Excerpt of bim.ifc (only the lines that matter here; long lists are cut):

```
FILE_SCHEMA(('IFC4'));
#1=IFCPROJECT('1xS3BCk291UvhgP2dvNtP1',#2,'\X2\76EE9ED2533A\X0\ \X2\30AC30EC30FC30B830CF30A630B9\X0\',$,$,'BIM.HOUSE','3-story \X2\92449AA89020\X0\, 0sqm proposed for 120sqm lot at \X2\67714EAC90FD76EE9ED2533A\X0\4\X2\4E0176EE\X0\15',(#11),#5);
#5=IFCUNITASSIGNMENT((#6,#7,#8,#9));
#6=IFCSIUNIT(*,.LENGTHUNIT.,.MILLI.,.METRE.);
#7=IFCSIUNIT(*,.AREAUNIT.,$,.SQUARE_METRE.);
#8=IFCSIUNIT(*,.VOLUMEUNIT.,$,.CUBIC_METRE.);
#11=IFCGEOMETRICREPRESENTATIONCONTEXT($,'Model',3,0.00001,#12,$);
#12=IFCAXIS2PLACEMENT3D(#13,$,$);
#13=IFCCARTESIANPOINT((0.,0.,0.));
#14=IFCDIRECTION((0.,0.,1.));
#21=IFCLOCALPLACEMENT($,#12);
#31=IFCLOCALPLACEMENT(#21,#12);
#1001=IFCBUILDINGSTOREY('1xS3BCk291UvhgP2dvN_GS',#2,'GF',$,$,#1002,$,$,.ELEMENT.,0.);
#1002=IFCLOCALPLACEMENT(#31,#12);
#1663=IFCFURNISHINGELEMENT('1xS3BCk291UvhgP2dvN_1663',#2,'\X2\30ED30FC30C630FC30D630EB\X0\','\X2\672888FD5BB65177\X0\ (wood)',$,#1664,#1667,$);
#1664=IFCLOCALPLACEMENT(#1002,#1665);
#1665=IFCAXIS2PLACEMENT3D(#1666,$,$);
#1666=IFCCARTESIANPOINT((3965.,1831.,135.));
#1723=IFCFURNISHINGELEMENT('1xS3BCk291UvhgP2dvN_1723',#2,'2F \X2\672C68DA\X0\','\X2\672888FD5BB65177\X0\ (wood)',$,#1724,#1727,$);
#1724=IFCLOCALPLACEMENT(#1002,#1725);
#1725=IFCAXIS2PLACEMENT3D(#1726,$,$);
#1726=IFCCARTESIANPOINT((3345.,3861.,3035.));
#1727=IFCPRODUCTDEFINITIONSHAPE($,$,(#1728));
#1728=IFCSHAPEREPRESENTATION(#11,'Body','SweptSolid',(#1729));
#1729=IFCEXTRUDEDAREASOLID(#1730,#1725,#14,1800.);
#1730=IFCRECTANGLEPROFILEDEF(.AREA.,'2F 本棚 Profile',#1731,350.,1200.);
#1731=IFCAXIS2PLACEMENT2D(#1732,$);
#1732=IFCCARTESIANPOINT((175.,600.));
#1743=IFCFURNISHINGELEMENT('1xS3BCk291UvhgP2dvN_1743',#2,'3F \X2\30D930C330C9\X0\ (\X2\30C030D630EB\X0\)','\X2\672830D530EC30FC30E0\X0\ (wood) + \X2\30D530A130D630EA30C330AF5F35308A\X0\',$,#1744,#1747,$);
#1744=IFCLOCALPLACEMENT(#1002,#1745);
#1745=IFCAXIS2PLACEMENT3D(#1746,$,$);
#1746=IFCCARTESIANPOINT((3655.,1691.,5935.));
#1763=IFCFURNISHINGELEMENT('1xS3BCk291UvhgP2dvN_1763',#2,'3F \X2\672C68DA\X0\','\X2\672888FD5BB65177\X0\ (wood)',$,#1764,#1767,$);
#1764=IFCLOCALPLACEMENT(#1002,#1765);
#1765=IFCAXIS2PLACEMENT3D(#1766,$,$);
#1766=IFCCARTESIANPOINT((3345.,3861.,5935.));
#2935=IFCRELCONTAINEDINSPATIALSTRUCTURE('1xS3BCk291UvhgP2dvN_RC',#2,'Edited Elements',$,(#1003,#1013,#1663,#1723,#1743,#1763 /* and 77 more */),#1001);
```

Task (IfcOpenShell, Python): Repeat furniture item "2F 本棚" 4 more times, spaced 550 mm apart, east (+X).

```python
import numpy as np
import ifcopenshell
import ifcopenshell.api.geometry
import ifcopenshell.api.root
import ifcopenshell.util.element
import ifcopenshell.util.placement

model = ifcopenshell.open("bim.ifc")


def reuse_history(source, copy):
    """copy_class also copies each property set's owner history, people and application; keep the originals."""
    for rel in copy.IsDefinedBy:
        if rel.is_a("IfcRelDefinesByProperties") and (history := rel.RelatingPropertyDefinition.OwnerHistory):
            rel.RelatingPropertyDefinition.OwnerHistory = source.OwnerHistory
            ifcopenshell.util.element.remove_deep2(model, history)


source = model.by_guid("1xS3BCk291UvhgP2dvN_1723")
base = ifcopenshell.util.placement.get_local_placement(source.ObjectPlacement)
step = np.array([1.0, 0.0, 0.0]) * 550.0

for i in range(1, 5):
    copy = ifcopenshell.api.root.copy_class(model, product=source)
    copy.Representation = ifcopenshell.util.element.copy_deep(
        model, source.Representation, exclude=["IfcGeometricRepresentationContext", "IfcRepresentationMap"]
    )
    reuse_history(source, copy)
    matrix = base.copy()
    matrix[:3, 3] += i * step
    print("added at", matrix[:3, 3].round(3) + 0.0)
    ifcopenshell.api.geometry.edit_object_placement(model, product=copy, matrix=matrix, is_si=False)

model.write("bim_edited.ifc")
```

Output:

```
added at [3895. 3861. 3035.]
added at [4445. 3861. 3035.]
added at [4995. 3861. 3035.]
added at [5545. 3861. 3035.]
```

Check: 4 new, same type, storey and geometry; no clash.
